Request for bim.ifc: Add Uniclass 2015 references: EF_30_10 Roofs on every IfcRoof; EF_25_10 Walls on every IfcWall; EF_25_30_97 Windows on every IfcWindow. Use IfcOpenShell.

First a look at what the model holds.

```python
import ifcopenshell

model = ifcopenshell.open("bim.ifc")
print(model.schema)
print("classifications:", [c.Name for c in model.by_type("IfcClassification")])
for ifc_class in ("IfcDoor", "IfcRoof", "IfcStair", "IfcWall", "IfcWindow"):
    print(ifc_class, len(model.by_type(ifc_class)))
```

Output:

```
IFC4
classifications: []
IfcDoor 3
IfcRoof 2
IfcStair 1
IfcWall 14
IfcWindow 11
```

```python
import ifcopenshell
import ifcopenshell.api.classification

model = ifcopenshell.open("bim.ifc")

system = ifcopenshell.api.classification.add_classification(model, classification="Uniclass 2015")

codes = {
    "IfcRoof": ("EF_30_10", "Roofs"),
    "IfcWall": ("EF_25_10", "Walls"),
    "IfcWindow": ("EF_25_30_97", "Windows"),
}
for ifc_class, (code, name) in codes.items():
    products = model.by_type(ifc_class)
    ifcopenshell.api.classification.add_reference(
        model, products=products, classification=system, identification=code, name=name
    )
    print(code, len(products))

model.write("bim_updated.ifc")
```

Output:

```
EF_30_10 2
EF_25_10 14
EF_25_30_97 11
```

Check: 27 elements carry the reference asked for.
